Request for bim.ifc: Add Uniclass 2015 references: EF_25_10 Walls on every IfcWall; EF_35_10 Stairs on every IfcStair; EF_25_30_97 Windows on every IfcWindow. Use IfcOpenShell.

First a look at what the model holds.

```python
import ifcopenshell

model = ifcopenshell.open("bim.ifc")
print(model.schema)
print("classifications:", [c.Name for c in model.by_type("IfcClassification")])
for ifc_class in ("IfcDoor", "IfcRoof", "IfcStair", "IfcWall", "IfcWindow"):
    print(ifc_class, len(model.by_type(ifc_class)))
```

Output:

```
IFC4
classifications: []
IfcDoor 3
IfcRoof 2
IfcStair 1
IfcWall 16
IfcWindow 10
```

```python
import ifcopenshell
import ifcopenshell.api.classification

model = ifcopenshell.open("bim.ifc")

system = ifcopenshell.api.classification.add_classification(model, classification="Uniclass 2015")

codes = {
    "IfcWall": ("EF_25_10", "Walls"),
    "IfcStair": ("EF_35_10", "Stairs"),
    "IfcWindow": ("EF_25_30_97", "Windows"),
}
for ifc_class, (code, name) in codes.items():
    products = model.by_type(ifc_class)
    ifcopenshell.api.classification.add_reference(
        model, products=products, classification=system, identification=code, name=name
    )
    print(code, len(products))

model.write("bim_rev.ifc")
```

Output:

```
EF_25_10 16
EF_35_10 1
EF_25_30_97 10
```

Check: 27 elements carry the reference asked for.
